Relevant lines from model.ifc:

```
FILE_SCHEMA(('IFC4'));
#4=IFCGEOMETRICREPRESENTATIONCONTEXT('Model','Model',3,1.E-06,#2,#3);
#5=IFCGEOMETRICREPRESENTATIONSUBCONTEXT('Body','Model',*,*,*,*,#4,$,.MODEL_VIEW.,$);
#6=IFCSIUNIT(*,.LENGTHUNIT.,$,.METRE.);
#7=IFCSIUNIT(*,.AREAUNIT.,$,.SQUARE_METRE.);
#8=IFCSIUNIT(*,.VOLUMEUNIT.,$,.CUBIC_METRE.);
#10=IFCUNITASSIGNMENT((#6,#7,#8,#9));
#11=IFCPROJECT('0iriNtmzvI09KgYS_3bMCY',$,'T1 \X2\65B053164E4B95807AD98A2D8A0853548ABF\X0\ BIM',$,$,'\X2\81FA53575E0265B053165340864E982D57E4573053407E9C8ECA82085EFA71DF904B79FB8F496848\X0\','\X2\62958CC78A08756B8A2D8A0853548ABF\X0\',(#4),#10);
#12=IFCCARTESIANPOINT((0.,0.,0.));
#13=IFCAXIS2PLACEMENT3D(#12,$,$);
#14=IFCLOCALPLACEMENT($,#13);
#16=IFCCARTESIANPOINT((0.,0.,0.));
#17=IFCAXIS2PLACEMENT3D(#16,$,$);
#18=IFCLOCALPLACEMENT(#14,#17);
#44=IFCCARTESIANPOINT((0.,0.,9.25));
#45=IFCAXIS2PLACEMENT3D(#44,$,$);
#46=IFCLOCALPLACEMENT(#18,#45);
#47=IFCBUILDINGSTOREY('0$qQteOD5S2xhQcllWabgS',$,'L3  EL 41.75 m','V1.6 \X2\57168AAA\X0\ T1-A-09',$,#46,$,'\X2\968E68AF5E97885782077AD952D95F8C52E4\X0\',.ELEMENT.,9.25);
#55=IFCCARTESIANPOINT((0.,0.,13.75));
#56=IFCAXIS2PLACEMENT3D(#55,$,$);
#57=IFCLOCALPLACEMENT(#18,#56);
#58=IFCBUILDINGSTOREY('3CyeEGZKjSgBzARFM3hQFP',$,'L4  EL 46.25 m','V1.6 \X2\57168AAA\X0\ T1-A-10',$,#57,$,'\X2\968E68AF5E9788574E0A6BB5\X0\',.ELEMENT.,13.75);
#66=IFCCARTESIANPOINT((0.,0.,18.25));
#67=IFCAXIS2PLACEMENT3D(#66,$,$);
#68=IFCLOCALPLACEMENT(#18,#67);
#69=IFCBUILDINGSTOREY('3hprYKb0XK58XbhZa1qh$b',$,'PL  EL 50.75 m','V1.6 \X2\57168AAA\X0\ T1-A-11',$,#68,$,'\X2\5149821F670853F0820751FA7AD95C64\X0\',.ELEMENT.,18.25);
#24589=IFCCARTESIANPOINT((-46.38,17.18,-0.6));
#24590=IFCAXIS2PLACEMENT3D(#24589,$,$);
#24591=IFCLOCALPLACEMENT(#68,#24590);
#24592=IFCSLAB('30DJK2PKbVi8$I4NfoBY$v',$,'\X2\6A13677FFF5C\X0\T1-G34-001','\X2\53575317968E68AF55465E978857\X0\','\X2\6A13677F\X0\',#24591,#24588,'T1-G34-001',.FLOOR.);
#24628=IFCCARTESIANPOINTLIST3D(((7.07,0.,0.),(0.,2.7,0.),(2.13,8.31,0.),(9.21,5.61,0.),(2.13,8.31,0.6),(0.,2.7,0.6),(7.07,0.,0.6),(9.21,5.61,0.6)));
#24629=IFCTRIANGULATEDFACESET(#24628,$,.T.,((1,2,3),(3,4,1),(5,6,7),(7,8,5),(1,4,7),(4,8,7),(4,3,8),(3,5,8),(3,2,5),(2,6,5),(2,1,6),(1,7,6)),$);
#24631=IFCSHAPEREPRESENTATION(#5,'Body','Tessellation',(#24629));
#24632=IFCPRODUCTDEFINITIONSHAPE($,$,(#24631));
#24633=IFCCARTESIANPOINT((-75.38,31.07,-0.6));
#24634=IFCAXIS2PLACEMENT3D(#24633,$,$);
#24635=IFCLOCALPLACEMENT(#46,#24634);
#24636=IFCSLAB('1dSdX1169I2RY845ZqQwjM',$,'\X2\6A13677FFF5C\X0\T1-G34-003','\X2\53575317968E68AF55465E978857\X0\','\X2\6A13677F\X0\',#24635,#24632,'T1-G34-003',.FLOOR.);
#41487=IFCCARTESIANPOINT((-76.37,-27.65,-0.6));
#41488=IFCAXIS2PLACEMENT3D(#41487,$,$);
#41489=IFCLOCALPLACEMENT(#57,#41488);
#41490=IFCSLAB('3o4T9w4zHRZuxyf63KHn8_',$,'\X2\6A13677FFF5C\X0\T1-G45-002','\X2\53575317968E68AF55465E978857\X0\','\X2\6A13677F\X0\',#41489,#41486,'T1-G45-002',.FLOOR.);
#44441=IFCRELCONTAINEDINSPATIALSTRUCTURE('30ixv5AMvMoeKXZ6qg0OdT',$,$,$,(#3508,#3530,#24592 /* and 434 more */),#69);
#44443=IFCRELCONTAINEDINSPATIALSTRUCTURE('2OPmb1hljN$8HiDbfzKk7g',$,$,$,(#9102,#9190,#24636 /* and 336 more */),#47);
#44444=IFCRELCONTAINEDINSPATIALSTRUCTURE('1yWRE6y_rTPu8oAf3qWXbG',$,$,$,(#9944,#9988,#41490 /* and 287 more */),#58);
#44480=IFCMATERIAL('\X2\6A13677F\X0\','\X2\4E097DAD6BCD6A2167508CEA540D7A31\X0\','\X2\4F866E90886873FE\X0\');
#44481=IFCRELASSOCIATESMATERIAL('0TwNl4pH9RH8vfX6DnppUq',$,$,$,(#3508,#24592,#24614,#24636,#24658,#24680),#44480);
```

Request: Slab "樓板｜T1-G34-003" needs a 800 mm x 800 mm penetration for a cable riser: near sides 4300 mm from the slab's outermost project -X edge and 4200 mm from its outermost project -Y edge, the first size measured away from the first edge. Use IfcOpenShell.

```python
import numpy as np
import ifcopenshell
import ifcopenshell.api.feature
import ifcopenshell.api.geometry
import ifcopenshell.api.root
import ifcopenshell.geom
import ifcopenshell.util.placement
import ifcopenshell.util.representation
import ifcopenshell.util.shape
import ifcopenshell.util.unit

model = ifcopenshell.open("model.ifc")
unit_scale = ifcopenshell.util.unit.calculate_unit_scale(model)
settings = ifcopenshell.geom.settings()


def volume(element):
    """Net volume in cubic metres, openings subtracted."""
    shape = ifcopenshell.geom.create_shape(settings, element)
    return ifcopenshell.util.shape.get_volume(shape.geometry)


slab = model.by_guid("1dSdX1169I2RY845ZqQwjM")
before = volume(slab)

# Extent in the slab's own axes, in metres. The edges named are its -X and -Y sides.
slab_shape = ifcopenshell.geom.create_shape(settings, slab)
vertices = ifcopenshell.util.shape.get_vertices(slab_shape.geometry)
x_min, y_min, bottom = vertices.min(axis=0)
top = vertices[:, 2].max()

opening = ifcopenshell.api.root.create_entity(model, ifc_class="IfcOpeningElement", name="Cable riser opening", predefined_type="OPENING")
context = ifcopenshell.util.representation.get_context(model, "Model", "Body", "MODEL_VIEW")
width, depth = 0.8, 0.8
outline = [(0.0, 0.0), (width, 0.0), (width, depth), (0.0, depth), (0.0, 0.0)]
# Overshoot both faces by 50 mm so the cut is clean.
shape = ifcopenshell.api.geometry.add_slab_representation(
    model, context=context, depth=top - bottom + 0.1, polyline=outline
)
ifcopenshell.api.geometry.assign_representation(model, product=opening, representation=shape)

matrix = ifcopenshell.util.placement.get_local_placement(slab.ObjectPlacement)
matrix[:, 3] = matrix @ np.append(np.array([x_min + 4.3, y_min + 4.2, bottom - 0.05]) / unit_scale, 1.0)
ifcopenshell.api.geometry.edit_object_placement(model, product=opening, matrix=matrix, is_si=False)
ifcopenshell.api.feature.add_feature(model, feature=opening, element=slab)

after = volume(slab)

print(f"slab volume {before:.3f} -> {after:.3f} m3")

model.write("model_v2.ifc")
```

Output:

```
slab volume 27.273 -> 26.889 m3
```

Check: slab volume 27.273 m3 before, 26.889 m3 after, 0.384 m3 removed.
